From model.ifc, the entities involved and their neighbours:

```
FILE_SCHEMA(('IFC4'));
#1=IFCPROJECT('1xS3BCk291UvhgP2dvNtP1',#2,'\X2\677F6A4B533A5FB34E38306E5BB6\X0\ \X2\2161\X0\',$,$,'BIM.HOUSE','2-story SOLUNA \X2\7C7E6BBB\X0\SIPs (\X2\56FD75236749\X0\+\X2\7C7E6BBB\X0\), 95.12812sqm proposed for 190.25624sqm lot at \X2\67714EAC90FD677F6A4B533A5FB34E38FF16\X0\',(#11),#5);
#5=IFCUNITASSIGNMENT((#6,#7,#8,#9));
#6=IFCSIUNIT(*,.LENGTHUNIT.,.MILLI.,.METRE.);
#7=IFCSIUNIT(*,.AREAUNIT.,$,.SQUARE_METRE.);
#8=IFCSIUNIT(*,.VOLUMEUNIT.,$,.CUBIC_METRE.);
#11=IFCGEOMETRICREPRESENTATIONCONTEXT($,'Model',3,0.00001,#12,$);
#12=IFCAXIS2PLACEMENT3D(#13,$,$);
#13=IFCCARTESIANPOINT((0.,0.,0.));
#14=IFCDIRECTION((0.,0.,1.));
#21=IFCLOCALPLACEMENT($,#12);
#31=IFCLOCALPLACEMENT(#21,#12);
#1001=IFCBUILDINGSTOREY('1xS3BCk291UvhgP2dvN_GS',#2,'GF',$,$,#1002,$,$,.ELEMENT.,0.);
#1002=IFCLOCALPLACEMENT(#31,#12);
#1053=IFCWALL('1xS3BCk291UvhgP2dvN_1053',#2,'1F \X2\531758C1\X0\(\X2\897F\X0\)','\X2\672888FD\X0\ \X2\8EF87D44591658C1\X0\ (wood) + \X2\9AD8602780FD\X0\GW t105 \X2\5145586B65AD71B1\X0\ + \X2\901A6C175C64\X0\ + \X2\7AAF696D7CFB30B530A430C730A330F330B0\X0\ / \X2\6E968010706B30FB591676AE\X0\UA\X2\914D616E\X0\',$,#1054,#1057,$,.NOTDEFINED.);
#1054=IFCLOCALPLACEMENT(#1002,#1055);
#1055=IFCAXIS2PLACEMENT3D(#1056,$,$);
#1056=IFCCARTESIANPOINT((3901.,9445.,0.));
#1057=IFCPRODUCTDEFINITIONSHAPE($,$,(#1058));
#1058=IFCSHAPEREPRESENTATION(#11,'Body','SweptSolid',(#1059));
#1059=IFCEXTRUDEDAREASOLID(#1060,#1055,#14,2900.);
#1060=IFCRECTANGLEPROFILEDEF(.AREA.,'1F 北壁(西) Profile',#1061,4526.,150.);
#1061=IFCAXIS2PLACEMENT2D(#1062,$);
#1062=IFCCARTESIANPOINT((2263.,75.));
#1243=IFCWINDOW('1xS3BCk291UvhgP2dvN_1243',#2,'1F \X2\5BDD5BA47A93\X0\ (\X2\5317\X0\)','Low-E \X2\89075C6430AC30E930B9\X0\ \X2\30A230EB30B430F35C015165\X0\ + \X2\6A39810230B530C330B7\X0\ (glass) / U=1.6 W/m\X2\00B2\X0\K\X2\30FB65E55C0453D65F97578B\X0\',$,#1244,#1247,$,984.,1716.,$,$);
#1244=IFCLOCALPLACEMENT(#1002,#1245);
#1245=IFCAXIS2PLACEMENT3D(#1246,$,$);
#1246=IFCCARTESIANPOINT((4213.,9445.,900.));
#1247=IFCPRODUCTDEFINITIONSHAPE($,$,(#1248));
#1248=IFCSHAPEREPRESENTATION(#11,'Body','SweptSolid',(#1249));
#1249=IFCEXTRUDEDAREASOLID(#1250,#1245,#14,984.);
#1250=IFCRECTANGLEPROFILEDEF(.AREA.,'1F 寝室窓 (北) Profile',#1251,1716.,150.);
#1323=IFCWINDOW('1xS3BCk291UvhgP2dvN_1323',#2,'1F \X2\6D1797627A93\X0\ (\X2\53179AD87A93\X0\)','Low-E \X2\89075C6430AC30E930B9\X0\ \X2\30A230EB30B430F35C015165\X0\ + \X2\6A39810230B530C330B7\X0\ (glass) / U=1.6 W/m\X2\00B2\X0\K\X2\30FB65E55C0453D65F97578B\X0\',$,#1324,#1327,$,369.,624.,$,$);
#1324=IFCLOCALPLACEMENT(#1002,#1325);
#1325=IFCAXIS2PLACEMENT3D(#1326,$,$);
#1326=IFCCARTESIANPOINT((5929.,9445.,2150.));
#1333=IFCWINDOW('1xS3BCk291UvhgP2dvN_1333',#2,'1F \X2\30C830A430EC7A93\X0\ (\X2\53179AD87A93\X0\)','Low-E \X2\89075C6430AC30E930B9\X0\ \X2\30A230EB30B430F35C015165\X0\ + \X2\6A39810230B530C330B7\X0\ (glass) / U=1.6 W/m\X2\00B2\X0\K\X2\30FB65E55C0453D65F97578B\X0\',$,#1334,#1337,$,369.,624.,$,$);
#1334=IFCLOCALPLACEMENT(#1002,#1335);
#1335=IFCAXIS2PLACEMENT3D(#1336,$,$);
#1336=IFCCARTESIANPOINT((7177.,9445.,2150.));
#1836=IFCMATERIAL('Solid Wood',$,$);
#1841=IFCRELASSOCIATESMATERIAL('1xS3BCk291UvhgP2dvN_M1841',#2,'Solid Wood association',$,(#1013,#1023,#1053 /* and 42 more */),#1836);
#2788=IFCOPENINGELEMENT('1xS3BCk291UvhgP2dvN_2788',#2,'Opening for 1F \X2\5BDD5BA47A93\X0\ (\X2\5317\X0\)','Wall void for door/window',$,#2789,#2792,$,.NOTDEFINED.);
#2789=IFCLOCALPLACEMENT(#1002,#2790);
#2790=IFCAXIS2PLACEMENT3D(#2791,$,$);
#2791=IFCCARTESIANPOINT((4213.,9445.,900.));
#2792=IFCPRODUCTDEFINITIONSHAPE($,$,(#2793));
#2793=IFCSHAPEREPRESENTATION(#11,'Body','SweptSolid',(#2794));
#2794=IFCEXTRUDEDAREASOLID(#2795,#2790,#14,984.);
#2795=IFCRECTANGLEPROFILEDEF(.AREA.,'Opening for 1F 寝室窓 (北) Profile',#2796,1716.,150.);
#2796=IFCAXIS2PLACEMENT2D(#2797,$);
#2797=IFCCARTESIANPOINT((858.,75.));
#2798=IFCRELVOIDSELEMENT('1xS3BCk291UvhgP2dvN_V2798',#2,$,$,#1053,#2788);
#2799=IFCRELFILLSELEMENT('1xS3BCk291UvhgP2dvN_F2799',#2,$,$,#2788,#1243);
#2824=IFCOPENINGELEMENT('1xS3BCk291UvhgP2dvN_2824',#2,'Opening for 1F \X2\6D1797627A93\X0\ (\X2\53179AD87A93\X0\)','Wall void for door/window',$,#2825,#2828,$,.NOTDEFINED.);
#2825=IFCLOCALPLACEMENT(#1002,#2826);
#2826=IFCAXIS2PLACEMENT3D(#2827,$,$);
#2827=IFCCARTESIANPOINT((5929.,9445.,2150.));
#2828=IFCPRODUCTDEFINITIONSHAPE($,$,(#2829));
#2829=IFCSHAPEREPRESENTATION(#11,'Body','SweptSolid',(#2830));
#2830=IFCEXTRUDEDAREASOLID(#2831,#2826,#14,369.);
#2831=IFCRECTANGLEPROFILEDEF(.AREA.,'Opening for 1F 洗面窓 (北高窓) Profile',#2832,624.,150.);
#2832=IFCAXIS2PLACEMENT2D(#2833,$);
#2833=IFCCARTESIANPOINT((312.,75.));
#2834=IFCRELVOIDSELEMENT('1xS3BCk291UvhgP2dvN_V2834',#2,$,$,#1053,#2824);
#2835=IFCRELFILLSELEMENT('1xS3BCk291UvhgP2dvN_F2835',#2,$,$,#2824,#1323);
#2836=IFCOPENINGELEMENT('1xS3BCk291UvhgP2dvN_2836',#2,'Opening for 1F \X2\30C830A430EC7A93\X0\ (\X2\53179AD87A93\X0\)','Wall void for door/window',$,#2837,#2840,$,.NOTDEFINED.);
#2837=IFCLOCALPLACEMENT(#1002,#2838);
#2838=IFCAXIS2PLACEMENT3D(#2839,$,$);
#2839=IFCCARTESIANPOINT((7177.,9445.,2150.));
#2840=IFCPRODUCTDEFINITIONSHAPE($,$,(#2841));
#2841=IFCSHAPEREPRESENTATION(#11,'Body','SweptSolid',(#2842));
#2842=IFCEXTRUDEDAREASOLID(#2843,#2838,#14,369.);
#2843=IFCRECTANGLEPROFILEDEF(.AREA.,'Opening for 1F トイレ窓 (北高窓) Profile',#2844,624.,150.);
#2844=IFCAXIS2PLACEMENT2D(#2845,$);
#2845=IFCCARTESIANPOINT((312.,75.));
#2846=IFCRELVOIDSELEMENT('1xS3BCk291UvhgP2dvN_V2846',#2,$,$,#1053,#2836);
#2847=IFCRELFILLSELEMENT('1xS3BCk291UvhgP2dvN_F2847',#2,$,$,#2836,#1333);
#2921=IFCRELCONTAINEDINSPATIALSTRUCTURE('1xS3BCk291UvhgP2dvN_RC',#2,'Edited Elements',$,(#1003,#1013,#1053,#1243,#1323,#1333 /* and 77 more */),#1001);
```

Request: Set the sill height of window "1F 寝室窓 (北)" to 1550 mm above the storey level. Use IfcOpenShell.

```python
import numpy as np
import ifcopenshell
import ifcopenshell.api.geometry
import ifcopenshell.geom
import ifcopenshell.util.element
import ifcopenshell.util.placement
import ifcopenshell.util.shape
import ifcopenshell.util.unit

model = ifcopenshell.open("model.ifc")
unit_scale = ifcopenshell.util.unit.calculate_unit_scale(model)

window = model.by_guid("1xS3BCk291UvhgP2dvN_1243")
opening = window.FillsVoids[0].RelatingOpeningElement
storey = ifcopenshell.util.element.get_container(window, ifc_class="IfcBuildingStorey")
level = ifcopenshell.util.placement.get_local_placement(storey.ObjectPlacement)[2, 3]

# The opening's origin need not be at the sill, so measure its lowest point.
shape = ifcopenshell.geom.create_shape(ifcopenshell.geom.settings(), opening)
bottom = ifcopenshell.util.shape.get_shape_bottom_elevation(shape, shape.geometry) / unit_scale
dz = level + 1550.0 - bottom

shift = np.array([0.0, 0.0, dz])
# The window is not placed relative to its opening, so move both.
for product in (opening, window):
    matrix = ifcopenshell.util.placement.get_local_placement(product.ObjectPlacement)
    matrix[:3, 3] += shift
    ifcopenshell.api.geometry.edit_object_placement(model, product=product, matrix=matrix, is_si=False)

print(f"moved by {dz * unit_scale:+.3f} m")

model.write("model_rev.ifc")
```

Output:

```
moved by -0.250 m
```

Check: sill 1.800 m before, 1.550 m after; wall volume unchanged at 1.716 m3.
